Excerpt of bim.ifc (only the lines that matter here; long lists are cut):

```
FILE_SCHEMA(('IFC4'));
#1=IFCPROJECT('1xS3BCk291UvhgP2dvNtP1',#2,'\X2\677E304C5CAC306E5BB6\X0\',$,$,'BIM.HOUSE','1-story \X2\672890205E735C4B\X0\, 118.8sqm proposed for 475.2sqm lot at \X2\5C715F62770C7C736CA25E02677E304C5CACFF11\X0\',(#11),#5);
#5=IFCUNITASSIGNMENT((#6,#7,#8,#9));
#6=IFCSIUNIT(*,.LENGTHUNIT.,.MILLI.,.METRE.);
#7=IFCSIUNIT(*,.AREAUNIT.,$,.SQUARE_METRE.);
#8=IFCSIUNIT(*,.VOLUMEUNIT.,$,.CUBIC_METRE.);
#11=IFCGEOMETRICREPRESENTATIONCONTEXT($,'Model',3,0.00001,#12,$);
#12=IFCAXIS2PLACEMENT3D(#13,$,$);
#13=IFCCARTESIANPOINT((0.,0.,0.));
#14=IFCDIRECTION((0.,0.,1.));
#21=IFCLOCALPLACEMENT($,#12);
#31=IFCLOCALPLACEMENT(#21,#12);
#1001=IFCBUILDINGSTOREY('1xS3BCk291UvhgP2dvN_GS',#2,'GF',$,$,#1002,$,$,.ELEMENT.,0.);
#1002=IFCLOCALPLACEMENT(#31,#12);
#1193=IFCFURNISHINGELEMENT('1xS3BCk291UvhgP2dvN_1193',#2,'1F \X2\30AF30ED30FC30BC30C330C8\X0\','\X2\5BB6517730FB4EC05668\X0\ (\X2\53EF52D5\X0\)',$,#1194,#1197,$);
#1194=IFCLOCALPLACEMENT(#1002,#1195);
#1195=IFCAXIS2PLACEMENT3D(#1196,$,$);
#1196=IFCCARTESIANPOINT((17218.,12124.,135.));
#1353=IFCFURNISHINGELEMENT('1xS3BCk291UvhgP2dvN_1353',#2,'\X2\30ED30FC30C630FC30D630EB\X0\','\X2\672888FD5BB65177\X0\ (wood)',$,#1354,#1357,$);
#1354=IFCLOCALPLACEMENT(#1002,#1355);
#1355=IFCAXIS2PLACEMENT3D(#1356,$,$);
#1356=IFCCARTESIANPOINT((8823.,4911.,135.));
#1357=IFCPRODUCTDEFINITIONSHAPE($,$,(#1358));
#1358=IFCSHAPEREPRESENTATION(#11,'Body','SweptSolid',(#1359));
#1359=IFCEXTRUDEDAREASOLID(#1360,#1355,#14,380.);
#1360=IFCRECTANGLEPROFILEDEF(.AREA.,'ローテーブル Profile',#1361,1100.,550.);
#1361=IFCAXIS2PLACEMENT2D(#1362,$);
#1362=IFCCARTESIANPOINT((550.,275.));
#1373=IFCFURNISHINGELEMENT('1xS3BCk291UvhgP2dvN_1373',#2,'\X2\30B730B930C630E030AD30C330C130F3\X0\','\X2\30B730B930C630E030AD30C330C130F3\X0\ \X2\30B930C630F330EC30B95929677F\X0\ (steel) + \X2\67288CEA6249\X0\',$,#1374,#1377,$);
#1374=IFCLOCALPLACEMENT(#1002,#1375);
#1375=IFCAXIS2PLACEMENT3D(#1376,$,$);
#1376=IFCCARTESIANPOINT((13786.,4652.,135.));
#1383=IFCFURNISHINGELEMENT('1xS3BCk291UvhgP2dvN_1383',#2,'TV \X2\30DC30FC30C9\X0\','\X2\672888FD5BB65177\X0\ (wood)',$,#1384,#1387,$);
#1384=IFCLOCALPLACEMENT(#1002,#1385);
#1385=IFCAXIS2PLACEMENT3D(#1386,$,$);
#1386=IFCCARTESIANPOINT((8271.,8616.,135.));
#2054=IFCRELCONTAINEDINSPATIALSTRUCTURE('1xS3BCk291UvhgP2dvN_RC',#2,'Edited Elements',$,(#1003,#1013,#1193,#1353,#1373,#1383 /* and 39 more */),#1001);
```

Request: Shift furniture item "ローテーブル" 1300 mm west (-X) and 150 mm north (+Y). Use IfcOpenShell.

```python
import ifcopenshell
import ifcopenshell.api.geometry
import ifcopenshell.util.placement

model = ifcopenshell.open("bim.ifc")

item = model.by_guid("1xS3BCk291UvhgP2dvN_1353")
matrix = ifcopenshell.util.placement.get_local_placement(item.ObjectPlacement)
matrix[0, 3] -= 1300.0
matrix[1, 3] += 150.0
ifcopenshell.api.geometry.edit_object_placement(model, product=item, matrix=matrix, is_si=False)

print(ifcopenshell.util.placement.get_local_placement(item.ObjectPlacement).round(3) + 0.0)

model.write("bim_updated.ifc")
```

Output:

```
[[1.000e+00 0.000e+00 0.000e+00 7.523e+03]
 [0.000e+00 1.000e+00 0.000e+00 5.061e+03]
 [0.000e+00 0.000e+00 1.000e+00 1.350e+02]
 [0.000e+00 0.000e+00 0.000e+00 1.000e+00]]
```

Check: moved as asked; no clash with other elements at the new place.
